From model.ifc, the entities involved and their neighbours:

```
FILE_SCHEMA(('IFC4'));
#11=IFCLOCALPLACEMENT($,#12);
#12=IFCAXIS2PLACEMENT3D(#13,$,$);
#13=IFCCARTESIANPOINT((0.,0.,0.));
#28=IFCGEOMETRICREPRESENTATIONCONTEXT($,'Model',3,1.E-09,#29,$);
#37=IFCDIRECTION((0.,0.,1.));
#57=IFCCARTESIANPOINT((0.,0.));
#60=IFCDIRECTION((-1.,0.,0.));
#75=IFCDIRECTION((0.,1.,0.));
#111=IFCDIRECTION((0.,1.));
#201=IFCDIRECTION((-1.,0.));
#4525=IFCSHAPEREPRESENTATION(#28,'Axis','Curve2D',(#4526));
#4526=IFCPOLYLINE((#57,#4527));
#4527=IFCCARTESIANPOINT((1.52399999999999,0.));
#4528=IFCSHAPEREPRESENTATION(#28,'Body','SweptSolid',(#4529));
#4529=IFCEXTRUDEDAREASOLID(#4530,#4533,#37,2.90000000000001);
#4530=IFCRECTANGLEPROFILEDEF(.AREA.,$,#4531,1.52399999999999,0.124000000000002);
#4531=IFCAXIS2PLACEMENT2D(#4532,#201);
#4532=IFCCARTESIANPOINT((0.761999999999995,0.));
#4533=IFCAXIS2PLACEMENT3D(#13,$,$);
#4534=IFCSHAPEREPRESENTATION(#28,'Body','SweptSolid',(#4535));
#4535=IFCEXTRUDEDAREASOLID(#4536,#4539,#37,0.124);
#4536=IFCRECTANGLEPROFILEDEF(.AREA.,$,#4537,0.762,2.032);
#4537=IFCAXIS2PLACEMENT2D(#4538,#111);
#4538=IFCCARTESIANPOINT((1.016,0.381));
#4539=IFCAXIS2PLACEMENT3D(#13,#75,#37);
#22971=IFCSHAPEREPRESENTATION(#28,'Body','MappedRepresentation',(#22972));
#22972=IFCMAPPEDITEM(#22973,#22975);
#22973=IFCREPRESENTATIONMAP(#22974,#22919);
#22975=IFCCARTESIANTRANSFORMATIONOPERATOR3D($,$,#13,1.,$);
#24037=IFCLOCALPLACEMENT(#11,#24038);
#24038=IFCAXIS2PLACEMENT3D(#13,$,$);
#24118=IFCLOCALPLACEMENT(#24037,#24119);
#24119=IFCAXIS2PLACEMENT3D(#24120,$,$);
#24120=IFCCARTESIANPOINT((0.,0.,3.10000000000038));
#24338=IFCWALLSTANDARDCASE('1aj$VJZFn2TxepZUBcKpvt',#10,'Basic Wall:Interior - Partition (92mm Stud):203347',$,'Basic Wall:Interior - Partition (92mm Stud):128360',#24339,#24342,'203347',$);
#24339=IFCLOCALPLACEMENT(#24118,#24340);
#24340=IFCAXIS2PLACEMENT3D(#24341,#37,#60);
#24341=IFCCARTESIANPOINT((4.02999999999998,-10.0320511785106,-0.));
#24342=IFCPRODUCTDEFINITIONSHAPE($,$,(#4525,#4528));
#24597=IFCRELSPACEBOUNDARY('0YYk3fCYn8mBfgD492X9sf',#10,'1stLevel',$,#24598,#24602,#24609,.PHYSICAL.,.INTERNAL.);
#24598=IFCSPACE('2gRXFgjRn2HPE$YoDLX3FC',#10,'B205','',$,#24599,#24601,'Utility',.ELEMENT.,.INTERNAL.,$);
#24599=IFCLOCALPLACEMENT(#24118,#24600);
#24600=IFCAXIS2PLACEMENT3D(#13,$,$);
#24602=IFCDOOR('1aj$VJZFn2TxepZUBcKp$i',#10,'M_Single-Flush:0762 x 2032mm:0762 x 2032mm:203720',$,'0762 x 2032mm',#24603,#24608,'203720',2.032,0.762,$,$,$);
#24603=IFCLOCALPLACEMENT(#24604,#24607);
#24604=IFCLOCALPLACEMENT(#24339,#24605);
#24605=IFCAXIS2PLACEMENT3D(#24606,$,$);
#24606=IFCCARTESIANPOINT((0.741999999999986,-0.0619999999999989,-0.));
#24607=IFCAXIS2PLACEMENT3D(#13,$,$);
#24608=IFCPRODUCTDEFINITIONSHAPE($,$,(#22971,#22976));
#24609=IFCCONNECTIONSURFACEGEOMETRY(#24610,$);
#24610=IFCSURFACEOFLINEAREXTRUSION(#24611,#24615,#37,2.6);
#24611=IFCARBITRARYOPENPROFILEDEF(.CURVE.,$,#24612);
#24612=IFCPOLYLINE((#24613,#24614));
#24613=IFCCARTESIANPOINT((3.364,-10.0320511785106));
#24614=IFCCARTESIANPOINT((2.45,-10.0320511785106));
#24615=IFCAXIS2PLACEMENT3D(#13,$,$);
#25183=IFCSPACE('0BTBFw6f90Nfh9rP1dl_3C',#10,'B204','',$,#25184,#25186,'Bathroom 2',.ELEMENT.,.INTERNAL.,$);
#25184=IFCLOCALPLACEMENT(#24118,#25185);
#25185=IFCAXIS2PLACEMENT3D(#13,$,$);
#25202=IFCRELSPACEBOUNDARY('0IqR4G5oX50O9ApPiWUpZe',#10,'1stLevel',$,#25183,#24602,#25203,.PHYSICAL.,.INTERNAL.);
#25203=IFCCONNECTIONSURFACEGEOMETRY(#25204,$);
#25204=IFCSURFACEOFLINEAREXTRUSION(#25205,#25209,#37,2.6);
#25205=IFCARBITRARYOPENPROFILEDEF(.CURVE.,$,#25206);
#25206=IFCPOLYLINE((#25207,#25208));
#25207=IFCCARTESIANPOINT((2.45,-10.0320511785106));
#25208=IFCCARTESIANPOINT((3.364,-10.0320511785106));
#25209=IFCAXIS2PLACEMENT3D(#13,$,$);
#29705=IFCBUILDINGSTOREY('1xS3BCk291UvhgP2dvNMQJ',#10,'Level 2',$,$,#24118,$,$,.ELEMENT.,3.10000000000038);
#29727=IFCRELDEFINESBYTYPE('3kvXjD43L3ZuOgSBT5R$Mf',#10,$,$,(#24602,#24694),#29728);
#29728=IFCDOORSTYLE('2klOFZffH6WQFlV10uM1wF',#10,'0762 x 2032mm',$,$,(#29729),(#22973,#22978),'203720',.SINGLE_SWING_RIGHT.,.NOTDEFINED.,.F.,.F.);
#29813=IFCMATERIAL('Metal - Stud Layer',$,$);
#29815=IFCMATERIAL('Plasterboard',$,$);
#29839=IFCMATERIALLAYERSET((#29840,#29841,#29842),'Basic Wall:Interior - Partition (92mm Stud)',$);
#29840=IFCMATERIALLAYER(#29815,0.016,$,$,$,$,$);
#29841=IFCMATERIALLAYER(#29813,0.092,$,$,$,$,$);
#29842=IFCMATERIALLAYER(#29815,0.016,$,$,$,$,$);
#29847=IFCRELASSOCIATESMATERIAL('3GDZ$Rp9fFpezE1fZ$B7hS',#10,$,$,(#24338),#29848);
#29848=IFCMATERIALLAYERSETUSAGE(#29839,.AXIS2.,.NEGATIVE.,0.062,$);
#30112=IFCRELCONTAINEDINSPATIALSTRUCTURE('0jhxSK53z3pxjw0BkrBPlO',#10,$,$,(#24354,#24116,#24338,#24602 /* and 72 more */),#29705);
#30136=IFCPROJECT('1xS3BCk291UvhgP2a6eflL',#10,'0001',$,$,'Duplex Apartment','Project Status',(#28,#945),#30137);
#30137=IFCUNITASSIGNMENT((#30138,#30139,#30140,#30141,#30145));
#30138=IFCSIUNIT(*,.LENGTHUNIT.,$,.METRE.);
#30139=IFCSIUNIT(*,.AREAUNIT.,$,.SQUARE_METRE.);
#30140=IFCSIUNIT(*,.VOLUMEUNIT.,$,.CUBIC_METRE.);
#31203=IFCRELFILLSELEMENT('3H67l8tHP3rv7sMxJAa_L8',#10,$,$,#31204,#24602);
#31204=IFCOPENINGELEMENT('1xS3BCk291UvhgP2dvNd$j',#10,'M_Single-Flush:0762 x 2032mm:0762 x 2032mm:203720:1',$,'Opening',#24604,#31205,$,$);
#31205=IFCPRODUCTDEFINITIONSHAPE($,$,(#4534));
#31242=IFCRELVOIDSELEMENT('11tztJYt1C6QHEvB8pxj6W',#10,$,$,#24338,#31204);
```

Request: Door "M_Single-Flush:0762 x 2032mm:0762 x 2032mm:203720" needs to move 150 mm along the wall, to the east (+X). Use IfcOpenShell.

```python
import numpy as np
import ifcopenshell
import ifcopenshell.api.geometry
import ifcopenshell.util.placement
import ifcopenshell.util.unit

model = ifcopenshell.open("model.ifc")
unit_scale = ifcopenshell.util.unit.calculate_unit_scale(model)

door = model.by_guid("1aj$VJZFn2TxepZUBcKp$i")
opening = door.FillsVoids[0].RelatingOpeningElement
wall = opening.VoidsElements[0].RelatingBuildingElement

wall_matrix = ifcopenshell.util.placement.get_local_placement(wall.ObjectPlacement)
shift = wall_matrix[:3, 0] * -0.15 / unit_scale
before = ifcopenshell.util.placement.get_local_placement(door.ObjectPlacement)[:3, 3].copy()

# The door is placed relative to its opening, so it follows when the opening moves.
matrix = ifcopenshell.util.placement.get_local_placement(opening.ObjectPlacement)
matrix[:3, 3] += shift
ifcopenshell.api.geometry.edit_object_placement(
    model, product=opening, matrix=matrix, is_si=False, should_transform_children=True
)

# Space boundary surfaces are stored in each space's coordinates; move them too.
for rel in door.ProvidesBoundaries:
    if not rel.ConnectionGeometry:
        continue
    surface = rel.ConnectionGeometry.SurfaceOnRelatingElement
    space_matrix = ifcopenshell.util.placement.get_local_placement(rel.RelatingSpace.ObjectPlacement)
    point = np.array(surface.Position.Location.Coordinates) + space_matrix[:3, :3].T @ shift
    surface.Position = model.createIfcAxis2Placement3D(
        model.createIfcCartesianPoint(point.tolist()), surface.Position.Axis, surface.Position.RefDirection
    )

after = ifcopenshell.util.placement.get_local_placement(door.ObjectPlacement)[:3, 3]
print("door moved by", (after - before).round(3) + 0.0)

model.write("model-out.ifc")
```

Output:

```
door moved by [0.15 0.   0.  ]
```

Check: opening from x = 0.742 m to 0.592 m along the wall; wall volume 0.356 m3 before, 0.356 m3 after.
